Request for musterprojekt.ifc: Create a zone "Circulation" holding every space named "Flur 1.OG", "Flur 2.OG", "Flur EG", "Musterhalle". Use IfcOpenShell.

First a look at what the model holds.

```python
import ifcopenshell

model = ifcopenshell.open("musterprojekt.ifc")
print(model.schema)
seen = {}
for space in model.by_type("IfcSpace"):
    seen[space.LongName] = seen.get(space.LongName, 0) + 1
for name, count in sorted(seen.items(), key=str):
    print(count, "x", name)
print("zones:", [z.Name for z in model.by_type("IfcZone")][:20])
```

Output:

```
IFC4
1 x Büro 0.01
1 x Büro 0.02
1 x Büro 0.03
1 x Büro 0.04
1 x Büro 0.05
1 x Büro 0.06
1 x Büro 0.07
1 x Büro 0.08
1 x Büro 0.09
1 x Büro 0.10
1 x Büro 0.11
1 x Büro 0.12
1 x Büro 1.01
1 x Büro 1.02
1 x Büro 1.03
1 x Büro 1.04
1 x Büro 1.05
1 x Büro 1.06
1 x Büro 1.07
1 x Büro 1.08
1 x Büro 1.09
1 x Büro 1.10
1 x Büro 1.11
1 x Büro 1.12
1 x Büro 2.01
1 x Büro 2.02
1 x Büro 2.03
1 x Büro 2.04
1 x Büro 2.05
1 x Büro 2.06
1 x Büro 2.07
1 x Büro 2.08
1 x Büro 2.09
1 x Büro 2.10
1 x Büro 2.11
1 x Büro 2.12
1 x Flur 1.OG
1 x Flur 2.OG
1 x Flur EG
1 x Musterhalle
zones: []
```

```python
import ifcopenshell
import ifcopenshell.api.group
import ifcopenshell.api.root

model = ifcopenshell.open("musterprojekt.ifc")

names = {"Flur 1.OG", "Flur 2.OG", "Flur EG", "Musterhalle"}
spaces = [s for s in model.by_type("IfcSpace") if s.LongName in names]

zone = ifcopenshell.api.root.create_entity(model, ifc_class="IfcZone", name="Circulation")
ifcopenshell.api.group.assign_group(model, products=spaces, group=zone)
print(len(spaces), "spaces in", zone.Name)

model.write("musterprojekt_rev.ifc")
```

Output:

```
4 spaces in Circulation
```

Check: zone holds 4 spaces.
